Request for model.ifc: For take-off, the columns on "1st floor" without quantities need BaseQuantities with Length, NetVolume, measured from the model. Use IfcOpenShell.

First a look at what the model holds.

```python
import ifcopenshell
import ifcopenshell.util.element
import ifcopenshell.util.unit

model = ifcopenshell.open("model.ifc")
print(model.schema)
for unit_type in ("LENGTHUNIT", "AREAUNIT", "VOLUMEUNIT"):
    print(unit_type, ifcopenshell.util.unit.calculate_unit_scale(model, unit_type))
storey = next(s for s in model.by_type("IfcBuildingStorey") if s.Name == "1st floor")
columns = [e for e in ifcopenshell.util.element.get_decomposition(storey) if e.is_a("IfcColumn")]
for e in sorted(columns, key=lambda e: e.id()):
    print(e.id(), e.is_a(), e.Name, list(ifcopenshell.util.element.get_psets(e, qtos_only=True)), sep=" | ")
```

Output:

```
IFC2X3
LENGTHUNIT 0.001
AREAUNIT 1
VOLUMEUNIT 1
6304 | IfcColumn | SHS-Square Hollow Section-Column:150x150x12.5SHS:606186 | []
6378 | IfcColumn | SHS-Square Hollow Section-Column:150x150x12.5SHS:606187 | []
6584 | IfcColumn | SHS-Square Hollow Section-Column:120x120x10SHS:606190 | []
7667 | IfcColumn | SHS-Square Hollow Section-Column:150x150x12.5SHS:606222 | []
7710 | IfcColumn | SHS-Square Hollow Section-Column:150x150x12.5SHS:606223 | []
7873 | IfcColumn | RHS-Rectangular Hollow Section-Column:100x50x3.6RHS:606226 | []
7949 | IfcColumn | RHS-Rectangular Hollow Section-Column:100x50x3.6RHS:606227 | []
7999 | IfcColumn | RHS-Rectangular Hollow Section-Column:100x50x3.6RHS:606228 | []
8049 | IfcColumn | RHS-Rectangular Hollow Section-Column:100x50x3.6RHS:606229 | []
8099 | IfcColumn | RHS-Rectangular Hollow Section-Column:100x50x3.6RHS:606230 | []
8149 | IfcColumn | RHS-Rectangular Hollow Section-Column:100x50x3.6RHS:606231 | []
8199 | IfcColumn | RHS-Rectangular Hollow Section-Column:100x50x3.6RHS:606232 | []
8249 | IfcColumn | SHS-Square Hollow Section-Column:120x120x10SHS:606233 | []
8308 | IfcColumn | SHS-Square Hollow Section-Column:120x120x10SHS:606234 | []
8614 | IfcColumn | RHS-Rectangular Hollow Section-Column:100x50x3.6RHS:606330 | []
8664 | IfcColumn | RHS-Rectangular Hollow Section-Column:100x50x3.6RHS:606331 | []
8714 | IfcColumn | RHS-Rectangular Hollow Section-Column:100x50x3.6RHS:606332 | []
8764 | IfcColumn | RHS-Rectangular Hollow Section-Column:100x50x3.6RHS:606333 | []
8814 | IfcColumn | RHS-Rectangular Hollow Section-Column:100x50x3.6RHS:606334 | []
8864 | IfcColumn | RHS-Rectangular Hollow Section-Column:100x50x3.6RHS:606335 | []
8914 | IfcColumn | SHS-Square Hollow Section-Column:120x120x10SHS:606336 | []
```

```python
import ifcopenshell
import ifcopenshell.api.pset
import ifcopenshell.geom
import ifcopenshell.util.element
import ifcopenshell.util.shape
import ifcopenshell.util.unit

model = ifcopenshell.open("model.ifc")
unit_scale = ifcopenshell.util.unit.calculate_unit_scale(model)
volume_scale = ifcopenshell.util.unit.calculate_unit_scale(model, "VOLUMEUNIT")
settings = ifcopenshell.geom.settings()

storey = next(s for s in model.by_type("IfcBuildingStorey") if s.Name == "1st floor")
columns = [e for e in ifcopenshell.util.element.get_decomposition(storey) if e.is_a("IfcColumn")]

for e in sorted(columns, key=lambda e: e.id()):
    if ifcopenshell.util.element.get_psets(e, qtos_only=True, should_inherit=False):
        continue
    # Geometry comes back in metres, in the element's own axes.
    shape = ifcopenshell.geom.create_shape(settings, e)
    values = {
        "Length": ifcopenshell.util.shape.get_z(shape.geometry) / unit_scale,
        "NetVolume": ifcopenshell.util.shape.get_volume(shape.geometry) / volume_scale,
    }
    qto = ifcopenshell.api.pset.add_qto(model, product=e, name="BaseQuantities")
    ifcopenshell.api.pset.edit_qto(model, qto=qto, properties=values)
    print(e.id(), {k: round(v, 3) for k, v in values.items()})

model.write("model-out.ifc")
```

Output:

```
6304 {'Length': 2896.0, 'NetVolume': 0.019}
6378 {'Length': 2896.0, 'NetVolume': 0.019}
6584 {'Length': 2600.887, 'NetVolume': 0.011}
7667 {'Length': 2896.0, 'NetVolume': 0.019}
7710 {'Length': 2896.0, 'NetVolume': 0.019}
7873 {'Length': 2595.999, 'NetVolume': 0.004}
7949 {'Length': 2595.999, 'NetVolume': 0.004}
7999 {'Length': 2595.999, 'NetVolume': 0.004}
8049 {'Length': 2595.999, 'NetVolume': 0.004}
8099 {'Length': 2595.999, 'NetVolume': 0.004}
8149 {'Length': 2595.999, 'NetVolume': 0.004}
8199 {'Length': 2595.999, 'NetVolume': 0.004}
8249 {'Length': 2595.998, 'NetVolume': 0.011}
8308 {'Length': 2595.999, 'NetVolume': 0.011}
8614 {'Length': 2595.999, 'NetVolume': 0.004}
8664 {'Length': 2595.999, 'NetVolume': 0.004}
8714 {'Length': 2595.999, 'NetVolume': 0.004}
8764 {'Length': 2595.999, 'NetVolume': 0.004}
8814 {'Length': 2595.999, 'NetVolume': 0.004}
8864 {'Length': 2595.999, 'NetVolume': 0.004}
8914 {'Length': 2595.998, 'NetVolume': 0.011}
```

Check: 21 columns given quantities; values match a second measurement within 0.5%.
